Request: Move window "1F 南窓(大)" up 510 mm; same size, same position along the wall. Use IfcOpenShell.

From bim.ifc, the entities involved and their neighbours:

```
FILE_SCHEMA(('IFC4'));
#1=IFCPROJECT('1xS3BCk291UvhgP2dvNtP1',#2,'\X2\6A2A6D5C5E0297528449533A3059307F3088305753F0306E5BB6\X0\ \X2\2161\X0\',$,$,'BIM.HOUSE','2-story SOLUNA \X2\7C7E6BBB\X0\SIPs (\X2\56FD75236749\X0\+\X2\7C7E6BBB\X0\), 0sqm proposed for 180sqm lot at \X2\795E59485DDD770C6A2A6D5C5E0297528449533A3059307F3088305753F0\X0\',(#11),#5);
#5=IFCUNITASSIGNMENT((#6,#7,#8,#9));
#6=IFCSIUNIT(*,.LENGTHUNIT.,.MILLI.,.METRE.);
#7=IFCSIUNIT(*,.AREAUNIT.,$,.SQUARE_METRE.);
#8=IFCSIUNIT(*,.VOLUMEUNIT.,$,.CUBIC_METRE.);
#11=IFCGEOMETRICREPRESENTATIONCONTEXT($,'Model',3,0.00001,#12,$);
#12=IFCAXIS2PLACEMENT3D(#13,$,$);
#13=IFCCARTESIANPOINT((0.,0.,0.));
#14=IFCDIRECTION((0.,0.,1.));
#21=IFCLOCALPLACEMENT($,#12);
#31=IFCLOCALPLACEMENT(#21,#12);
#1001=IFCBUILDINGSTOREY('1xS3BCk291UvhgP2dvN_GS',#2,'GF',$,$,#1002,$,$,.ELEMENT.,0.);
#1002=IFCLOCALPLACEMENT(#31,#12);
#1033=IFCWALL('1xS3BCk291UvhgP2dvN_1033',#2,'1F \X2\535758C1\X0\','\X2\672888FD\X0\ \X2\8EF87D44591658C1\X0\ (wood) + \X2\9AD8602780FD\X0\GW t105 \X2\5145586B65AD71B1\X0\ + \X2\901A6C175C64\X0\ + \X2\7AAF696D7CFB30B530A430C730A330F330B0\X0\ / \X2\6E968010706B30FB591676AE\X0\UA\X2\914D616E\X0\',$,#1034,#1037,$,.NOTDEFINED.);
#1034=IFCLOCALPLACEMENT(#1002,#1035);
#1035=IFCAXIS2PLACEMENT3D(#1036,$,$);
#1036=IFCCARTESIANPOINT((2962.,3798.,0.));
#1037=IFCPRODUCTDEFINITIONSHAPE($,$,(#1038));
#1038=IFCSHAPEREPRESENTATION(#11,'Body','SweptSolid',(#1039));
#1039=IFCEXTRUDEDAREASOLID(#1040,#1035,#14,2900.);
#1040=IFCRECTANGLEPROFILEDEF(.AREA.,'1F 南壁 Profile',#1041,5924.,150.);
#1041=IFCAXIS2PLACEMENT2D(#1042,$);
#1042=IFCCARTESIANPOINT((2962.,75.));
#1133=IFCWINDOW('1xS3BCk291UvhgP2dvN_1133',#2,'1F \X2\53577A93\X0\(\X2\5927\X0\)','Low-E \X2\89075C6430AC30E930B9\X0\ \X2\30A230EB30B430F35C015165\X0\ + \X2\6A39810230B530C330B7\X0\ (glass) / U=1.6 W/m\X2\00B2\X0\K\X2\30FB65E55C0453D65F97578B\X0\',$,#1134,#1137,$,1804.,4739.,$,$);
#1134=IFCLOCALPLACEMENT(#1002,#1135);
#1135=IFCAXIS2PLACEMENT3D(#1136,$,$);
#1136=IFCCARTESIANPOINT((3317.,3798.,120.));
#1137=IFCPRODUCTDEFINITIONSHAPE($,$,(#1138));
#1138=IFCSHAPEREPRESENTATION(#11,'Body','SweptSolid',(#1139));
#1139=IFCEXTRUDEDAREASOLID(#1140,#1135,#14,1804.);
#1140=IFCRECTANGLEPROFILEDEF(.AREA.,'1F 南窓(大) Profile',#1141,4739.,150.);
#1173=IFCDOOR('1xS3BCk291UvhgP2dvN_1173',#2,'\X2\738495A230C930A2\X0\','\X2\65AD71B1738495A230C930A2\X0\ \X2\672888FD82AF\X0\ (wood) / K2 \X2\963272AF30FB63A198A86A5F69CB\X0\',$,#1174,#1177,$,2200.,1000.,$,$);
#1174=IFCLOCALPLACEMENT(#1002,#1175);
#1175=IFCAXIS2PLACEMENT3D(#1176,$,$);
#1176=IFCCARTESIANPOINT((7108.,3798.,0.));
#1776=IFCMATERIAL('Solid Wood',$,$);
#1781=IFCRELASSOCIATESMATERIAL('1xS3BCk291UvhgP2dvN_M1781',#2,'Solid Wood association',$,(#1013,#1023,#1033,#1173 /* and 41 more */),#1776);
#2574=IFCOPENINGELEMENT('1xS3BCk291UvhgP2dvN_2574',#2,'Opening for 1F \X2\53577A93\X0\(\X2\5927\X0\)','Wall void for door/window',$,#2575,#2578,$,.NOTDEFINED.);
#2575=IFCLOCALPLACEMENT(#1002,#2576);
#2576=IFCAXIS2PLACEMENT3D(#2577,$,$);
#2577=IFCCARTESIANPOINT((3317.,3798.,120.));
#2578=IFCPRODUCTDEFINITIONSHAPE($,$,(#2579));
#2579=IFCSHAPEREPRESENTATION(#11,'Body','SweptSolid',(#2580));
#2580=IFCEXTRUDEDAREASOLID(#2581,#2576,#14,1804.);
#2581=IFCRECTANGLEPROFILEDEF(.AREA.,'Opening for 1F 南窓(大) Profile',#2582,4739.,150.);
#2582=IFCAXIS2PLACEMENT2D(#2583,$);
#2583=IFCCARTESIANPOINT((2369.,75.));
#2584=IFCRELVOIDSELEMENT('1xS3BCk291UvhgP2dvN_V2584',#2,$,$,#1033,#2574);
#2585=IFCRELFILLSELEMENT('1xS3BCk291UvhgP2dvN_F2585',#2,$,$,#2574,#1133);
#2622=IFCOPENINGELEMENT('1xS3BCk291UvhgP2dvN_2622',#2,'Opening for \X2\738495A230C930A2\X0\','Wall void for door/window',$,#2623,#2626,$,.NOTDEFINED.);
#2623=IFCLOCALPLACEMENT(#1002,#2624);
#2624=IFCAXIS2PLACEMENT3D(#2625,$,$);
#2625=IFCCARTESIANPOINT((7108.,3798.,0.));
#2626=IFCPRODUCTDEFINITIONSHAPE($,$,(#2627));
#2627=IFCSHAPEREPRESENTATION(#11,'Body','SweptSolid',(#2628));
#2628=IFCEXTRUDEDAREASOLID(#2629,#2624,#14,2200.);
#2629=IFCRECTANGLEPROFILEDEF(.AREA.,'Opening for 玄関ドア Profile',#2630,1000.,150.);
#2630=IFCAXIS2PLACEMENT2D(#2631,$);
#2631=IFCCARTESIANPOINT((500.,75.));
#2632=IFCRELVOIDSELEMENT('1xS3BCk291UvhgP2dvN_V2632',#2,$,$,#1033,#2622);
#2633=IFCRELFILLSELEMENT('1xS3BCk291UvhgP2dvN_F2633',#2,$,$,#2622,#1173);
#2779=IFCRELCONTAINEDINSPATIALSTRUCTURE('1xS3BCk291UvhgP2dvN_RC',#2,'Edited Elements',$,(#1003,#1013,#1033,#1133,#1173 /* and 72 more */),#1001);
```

```python
import numpy as np
import ifcopenshell
import ifcopenshell.api.geometry
import ifcopenshell.util.placement
import ifcopenshell.util.unit

model = ifcopenshell.open("bim.ifc")
unit_scale = ifcopenshell.util.unit.calculate_unit_scale(model)

window = model.by_guid("1xS3BCk291UvhgP2dvN_1133")
opening = window.FillsVoids[0].RelatingOpeningElement
dz = 510.0

shift = np.array([0.0, 0.0, dz])
# The window is not placed relative to its opening, so move both.
for product in (opening, window):
    matrix = ifcopenshell.util.placement.get_local_placement(product.ObjectPlacement)
    matrix[:3, 3] += shift
    ifcopenshell.api.geometry.edit_object_placement(model, product=product, matrix=matrix, is_si=False)

print(f"moved by {dz * unit_scale:+.3f} m")

model.write("bim_updated.ifc")
```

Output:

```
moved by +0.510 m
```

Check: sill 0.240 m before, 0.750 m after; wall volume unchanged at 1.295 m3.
